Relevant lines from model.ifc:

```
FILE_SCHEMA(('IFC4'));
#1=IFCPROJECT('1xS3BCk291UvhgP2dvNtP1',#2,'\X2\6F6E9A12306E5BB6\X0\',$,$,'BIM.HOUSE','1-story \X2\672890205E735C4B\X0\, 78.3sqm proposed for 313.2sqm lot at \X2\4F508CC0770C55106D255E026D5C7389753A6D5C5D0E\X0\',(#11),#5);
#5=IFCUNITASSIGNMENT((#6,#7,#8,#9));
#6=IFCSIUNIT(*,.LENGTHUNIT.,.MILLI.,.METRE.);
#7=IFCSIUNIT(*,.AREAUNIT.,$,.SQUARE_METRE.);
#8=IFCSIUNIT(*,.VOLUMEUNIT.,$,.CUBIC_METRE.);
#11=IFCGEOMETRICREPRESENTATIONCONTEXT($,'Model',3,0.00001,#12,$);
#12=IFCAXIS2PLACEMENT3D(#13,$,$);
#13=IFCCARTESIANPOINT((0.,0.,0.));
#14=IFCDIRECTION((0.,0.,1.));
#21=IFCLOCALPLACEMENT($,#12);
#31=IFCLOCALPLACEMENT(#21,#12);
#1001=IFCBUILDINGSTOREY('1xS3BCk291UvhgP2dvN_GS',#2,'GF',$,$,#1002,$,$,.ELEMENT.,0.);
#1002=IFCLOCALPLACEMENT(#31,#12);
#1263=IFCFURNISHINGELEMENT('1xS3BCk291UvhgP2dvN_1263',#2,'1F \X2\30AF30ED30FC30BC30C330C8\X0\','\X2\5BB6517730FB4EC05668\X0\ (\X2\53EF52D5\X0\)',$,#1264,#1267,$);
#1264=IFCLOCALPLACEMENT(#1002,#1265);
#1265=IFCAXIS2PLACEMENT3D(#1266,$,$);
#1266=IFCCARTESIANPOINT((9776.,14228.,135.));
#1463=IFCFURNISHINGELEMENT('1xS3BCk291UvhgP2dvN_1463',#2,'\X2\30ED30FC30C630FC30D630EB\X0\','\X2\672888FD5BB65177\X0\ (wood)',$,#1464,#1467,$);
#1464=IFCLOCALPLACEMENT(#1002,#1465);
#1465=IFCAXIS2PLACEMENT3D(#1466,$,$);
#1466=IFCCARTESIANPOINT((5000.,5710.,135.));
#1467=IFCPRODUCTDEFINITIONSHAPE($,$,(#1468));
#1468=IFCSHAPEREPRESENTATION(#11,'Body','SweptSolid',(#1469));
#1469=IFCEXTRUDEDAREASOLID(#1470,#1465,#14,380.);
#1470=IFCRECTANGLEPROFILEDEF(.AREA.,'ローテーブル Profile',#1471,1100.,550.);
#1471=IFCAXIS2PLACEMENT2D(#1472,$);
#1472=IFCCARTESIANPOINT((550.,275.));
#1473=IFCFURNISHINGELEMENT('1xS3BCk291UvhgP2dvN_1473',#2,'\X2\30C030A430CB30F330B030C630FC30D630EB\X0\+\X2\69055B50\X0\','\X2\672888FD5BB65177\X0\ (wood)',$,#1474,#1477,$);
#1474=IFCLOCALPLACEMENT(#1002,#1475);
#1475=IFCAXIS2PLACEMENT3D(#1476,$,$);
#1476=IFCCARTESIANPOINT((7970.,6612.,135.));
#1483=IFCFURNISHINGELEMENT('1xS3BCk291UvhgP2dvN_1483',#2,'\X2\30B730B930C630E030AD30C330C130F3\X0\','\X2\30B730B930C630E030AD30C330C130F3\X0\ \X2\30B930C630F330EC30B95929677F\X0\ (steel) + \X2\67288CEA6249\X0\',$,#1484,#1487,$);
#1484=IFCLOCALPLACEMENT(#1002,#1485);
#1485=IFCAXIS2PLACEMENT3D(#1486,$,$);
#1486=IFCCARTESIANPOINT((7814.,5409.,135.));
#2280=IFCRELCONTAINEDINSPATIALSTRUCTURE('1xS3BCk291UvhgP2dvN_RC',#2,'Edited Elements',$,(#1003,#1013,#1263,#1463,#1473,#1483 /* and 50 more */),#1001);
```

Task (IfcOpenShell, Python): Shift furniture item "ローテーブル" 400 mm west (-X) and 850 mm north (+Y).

```python
import ifcopenshell
import ifcopenshell.api.geometry
import ifcopenshell.util.placement
import ifcopenshell.util.unit

model = ifcopenshell.open("model.ifc")
unit_scale = ifcopenshell.util.unit.calculate_unit_scale(model)

item = model.by_guid("1xS3BCk291UvhgP2dvN_1463")
matrix = ifcopenshell.util.placement.get_local_placement(item.ObjectPlacement)
matrix[0, 3] -= 0.4 / unit_scale
matrix[1, 3] += 0.85 / unit_scale
ifcopenshell.api.geometry.edit_object_placement(model, product=item, matrix=matrix, is_si=False)

print(ifcopenshell.util.placement.get_local_placement(item.ObjectPlacement).round(3) + 0.0)

model.write("model_updated.ifc")
```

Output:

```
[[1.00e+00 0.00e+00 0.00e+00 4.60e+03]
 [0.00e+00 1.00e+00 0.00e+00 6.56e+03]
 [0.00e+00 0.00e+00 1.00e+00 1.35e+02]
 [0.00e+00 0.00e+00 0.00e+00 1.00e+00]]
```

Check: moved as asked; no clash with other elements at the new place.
